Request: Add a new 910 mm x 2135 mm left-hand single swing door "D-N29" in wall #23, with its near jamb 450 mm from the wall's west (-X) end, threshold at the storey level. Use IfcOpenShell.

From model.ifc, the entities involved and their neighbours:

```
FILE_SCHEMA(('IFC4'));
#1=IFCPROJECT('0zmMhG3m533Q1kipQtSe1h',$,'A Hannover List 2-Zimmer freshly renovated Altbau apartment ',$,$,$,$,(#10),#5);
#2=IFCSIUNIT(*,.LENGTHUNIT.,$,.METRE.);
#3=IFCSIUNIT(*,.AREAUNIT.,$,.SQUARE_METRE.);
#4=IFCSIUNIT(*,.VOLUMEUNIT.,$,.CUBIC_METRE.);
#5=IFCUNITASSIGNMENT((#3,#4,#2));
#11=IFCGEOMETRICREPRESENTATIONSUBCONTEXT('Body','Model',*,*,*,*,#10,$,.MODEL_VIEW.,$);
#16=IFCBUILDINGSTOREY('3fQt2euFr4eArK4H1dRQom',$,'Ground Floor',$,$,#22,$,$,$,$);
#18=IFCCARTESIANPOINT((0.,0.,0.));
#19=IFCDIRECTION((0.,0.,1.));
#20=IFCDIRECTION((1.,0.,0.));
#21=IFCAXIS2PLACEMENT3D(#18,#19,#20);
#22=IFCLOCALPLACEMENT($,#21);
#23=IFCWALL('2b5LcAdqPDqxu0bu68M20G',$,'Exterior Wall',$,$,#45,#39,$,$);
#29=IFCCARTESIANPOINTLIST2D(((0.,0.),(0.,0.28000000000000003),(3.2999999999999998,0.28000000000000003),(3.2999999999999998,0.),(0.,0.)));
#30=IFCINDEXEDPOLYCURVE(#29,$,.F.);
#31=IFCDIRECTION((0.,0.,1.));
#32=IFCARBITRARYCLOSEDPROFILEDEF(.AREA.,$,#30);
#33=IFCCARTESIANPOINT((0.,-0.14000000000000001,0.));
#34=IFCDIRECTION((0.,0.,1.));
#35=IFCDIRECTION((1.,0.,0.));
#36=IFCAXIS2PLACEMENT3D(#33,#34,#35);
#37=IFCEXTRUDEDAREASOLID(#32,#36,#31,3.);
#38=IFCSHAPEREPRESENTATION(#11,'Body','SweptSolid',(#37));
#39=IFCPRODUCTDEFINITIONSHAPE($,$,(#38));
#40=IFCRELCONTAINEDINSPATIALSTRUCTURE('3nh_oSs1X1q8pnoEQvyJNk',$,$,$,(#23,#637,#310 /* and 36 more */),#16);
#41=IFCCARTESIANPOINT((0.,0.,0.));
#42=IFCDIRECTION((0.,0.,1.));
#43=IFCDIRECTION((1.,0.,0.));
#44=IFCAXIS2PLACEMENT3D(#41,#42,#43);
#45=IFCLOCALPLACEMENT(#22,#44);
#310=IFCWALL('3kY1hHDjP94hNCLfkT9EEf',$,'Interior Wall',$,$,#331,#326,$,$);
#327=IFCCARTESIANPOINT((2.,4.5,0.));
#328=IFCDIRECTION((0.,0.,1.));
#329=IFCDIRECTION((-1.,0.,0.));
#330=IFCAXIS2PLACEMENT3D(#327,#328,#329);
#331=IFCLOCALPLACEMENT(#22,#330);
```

```python
import numpy as np
import ifcopenshell
import ifcopenshell.api.feature
import ifcopenshell.api.geometry
import ifcopenshell.api.root
import ifcopenshell.api.spatial
import ifcopenshell.geom
import ifcopenshell.util.element
import ifcopenshell.util.placement
import ifcopenshell.util.representation
import ifcopenshell.util.shape
import ifcopenshell.util.unit

model = ifcopenshell.open("model.ifc")
unit_scale = ifcopenshell.util.unit.calculate_unit_scale(model)
settings = ifcopenshell.geom.settings()


def volume(element):
    """Net volume in cubic metres, openings subtracted."""
    shape = ifcopenshell.geom.create_shape(settings, element)
    return ifcopenshell.util.shape.get_volume(shape.geometry)


wall = model.by_id(23)
storey = ifcopenshell.util.element.get_container(wall, ifc_class="IfcBuildingStorey")
context = ifcopenshell.util.representation.get_context(model, "Model", "Body", "MODEL_VIEW")
before = volume(wall)

width, height, from_end, sill = 0.91, 2.135, 0.45, 0.0  # metres

# The wall runs along its own X axis, and the end named is its -X end.
wall_shape = ifcopenshell.geom.create_shape(settings, wall)
x, y, z = ifcopenshell.util.shape.get_vertices(wall_shape.geometry).T
start = x.min() + from_end
face, thickness = float(y.min()), float(y.max() - y.min())
wall_matrix = ifcopenshell.util.placement.get_local_placement(wall.ObjectPlacement)
level = ifcopenshell.util.placement.get_local_placement(storey.ObjectPlacement)[2, 3]


def in_wall(x, y):
    """Placement at x, y metres in the wall's axes, at sill height."""
    matrix = wall_matrix.copy()
    matrix[:, 3] = wall_matrix @ np.array([x / unit_scale, y / unit_scale, 0.0, 1.0])
    matrix[2, 3] = level + sill / unit_scale
    return matrix


# Opening: a box that overshoots both wall faces by 50 mm.
opening = ifcopenshell.api.root.create_entity(model, ifc_class="IfcOpeningElement", predefined_type="OPENING")
box = ifcopenshell.api.geometry.add_wall_representation(
    model, context=context, length=width, height=height, thickness=thickness + 0.1
)
ifcopenshell.api.geometry.assign_representation(model, product=opening, representation=box)
ifcopenshell.api.geometry.edit_object_placement(model, product=opening, matrix=in_wall(start, face - 0.05), is_si=False)
ifcopenshell.api.feature.add_feature(model, feature=opening, element=wall)

door = ifcopenshell.api.root.create_entity(model, ifc_class="IfcDoor", name="D-N29", predefined_type="DOOR")
door.OverallWidth, door.OverallHeight = width / unit_scale, height / unit_scale
door.OperationType = "SINGLE_SWING_LEFT"
body = ifcopenshell.api.geometry.add_door_representation(
    model,
    context=context,
    overall_width=door.OverallWidth,
    overall_height=door.OverallHeight,
    operation_type="SINGLE_SWING_LEFT",
    lining_properties={"LiningDepth": thickness / unit_scale, "ThresholdDepth": thickness / unit_scale},
)
ifcopenshell.api.geometry.assign_representation(model, product=door, representation=body)
ifcopenshell.api.spatial.assign_container(model, products=[door], relating_structure=storey)
ifcopenshell.api.feature.add_filling(model, opening=opening, element=door)

# The lining spans the wall, so the door starts at the wall face.
ifcopenshell.api.geometry.edit_object_placement(model, product=door, matrix=in_wall(start, face), is_si=False)

after = volume(wall)

print(f"wall volume {before:.3f} -> {after:.3f} m3")

model.write("model_edited.ifc")
```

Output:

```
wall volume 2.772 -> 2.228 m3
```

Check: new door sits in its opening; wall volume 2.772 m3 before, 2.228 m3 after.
